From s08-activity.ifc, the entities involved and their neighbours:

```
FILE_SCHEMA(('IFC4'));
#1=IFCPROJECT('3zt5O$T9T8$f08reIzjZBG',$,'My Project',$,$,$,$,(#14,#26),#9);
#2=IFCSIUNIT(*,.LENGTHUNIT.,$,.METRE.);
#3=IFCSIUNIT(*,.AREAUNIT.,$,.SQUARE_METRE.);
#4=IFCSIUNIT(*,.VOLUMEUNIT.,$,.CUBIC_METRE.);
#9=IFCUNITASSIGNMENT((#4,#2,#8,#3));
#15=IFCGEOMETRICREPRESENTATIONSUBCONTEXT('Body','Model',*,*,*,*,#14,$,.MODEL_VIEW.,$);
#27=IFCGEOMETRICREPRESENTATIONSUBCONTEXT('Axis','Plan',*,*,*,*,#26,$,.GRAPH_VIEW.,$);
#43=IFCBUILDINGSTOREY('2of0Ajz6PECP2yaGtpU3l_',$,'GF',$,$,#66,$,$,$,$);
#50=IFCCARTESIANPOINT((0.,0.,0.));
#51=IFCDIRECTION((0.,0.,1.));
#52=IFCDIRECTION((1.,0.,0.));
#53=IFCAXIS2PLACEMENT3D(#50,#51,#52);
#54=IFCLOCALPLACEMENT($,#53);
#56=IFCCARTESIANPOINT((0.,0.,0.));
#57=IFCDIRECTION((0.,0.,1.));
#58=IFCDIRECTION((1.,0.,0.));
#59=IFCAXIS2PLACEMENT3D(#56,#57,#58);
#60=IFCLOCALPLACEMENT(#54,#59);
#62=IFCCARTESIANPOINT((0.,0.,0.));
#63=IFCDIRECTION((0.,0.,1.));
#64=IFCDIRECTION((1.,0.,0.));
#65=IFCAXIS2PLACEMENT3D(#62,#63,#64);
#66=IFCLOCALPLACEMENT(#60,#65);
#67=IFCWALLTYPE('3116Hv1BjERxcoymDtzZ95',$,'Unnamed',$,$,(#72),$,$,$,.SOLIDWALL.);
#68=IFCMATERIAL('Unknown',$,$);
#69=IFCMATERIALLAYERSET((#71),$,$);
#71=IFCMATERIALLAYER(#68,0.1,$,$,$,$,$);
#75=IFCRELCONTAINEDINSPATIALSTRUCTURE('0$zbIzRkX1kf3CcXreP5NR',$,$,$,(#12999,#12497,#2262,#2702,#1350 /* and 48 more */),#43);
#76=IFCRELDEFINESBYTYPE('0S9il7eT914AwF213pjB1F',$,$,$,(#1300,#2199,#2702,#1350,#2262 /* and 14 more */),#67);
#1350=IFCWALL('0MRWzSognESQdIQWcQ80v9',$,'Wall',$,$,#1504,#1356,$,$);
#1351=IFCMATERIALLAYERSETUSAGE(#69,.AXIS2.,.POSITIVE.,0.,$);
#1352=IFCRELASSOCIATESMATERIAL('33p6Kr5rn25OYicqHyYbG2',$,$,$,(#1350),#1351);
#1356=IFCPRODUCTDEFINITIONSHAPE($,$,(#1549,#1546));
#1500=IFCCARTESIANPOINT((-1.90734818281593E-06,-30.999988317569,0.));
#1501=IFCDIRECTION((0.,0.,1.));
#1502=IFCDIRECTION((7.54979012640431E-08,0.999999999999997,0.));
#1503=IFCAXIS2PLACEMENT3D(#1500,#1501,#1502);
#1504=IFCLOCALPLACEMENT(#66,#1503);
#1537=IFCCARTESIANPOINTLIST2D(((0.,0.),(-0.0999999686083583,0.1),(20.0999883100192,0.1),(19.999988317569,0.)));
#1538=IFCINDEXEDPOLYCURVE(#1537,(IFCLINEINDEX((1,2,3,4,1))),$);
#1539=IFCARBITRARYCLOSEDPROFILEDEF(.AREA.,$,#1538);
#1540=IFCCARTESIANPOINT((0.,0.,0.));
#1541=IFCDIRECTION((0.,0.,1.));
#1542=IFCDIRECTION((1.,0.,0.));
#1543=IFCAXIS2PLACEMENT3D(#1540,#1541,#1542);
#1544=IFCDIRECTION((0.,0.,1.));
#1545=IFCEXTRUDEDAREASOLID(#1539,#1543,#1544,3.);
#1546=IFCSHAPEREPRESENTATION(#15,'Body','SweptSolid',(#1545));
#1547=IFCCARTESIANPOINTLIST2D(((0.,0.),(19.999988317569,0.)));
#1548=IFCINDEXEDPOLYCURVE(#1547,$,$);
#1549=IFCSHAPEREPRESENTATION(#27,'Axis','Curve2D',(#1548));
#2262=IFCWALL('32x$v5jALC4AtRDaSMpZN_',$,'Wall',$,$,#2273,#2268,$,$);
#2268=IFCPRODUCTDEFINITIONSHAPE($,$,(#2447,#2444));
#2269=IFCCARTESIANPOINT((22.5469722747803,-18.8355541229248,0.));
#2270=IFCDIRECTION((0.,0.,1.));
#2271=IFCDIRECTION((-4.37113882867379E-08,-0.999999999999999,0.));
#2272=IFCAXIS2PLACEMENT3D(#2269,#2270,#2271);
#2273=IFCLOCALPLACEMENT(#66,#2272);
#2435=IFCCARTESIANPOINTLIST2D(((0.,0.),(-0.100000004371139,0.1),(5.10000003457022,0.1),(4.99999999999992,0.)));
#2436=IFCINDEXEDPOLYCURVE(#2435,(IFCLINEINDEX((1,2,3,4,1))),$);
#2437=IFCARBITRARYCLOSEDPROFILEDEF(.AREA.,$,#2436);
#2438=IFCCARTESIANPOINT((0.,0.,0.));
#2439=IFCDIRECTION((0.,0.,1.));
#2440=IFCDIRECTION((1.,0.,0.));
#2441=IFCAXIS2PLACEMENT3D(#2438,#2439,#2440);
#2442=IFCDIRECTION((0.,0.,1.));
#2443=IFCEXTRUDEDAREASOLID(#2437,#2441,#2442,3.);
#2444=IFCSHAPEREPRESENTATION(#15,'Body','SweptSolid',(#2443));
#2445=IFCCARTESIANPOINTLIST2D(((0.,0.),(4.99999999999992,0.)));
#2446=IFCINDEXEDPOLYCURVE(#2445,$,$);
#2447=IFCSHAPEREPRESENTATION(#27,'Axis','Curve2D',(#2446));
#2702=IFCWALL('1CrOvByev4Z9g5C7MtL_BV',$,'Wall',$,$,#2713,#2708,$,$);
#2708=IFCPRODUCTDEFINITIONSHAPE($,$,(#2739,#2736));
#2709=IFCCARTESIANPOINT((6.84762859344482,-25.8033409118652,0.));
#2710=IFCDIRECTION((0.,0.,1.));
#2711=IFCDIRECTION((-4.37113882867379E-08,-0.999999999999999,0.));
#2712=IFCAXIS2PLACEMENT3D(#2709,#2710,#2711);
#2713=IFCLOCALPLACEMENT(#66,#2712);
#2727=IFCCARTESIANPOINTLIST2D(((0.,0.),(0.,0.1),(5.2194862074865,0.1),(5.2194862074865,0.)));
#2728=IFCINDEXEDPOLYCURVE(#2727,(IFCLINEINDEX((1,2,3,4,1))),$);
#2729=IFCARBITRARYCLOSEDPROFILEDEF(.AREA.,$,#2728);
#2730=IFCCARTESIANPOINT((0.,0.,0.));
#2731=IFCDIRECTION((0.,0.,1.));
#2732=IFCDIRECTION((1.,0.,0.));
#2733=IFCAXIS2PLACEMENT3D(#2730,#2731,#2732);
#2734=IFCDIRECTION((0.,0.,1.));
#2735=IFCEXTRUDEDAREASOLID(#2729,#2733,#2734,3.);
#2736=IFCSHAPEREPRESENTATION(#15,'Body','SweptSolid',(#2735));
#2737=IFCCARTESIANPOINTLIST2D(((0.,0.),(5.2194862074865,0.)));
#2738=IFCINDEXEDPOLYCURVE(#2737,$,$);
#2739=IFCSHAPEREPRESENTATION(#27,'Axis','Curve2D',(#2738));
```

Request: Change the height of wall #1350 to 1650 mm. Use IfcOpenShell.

```python
import ifcopenshell
import ifcopenshell.geom
import ifcopenshell.util.representation
import ifcopenshell.util.shape

model = ifcopenshell.open("s08-activity.ifc")
settings = ifcopenshell.geom.settings()


def volume(element):
    """Net volume in cubic metres, openings subtracted."""
    shape = ifcopenshell.geom.create_shape(settings, element)
    return ifcopenshell.util.shape.get_volume(shape.geometry)


wall = model.by_guid("0MRWzSognESQdIQWcQ80v9")
before = volume(wall)

body = ifcopenshell.util.representation.get_representation(wall, "Model", "Body")
solid = body.Items[0]
old_height = solid.Depth
solid.Depth = 1.65
after = volume(wall)

print(f"height {old_height:g} -> {solid.Depth:g}, volume {before:.3f} -> {after:.3f} m3")

model.write("s08-activity_edited.ifc")
```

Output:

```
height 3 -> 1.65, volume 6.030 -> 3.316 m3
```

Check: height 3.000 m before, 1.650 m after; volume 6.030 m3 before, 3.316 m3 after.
